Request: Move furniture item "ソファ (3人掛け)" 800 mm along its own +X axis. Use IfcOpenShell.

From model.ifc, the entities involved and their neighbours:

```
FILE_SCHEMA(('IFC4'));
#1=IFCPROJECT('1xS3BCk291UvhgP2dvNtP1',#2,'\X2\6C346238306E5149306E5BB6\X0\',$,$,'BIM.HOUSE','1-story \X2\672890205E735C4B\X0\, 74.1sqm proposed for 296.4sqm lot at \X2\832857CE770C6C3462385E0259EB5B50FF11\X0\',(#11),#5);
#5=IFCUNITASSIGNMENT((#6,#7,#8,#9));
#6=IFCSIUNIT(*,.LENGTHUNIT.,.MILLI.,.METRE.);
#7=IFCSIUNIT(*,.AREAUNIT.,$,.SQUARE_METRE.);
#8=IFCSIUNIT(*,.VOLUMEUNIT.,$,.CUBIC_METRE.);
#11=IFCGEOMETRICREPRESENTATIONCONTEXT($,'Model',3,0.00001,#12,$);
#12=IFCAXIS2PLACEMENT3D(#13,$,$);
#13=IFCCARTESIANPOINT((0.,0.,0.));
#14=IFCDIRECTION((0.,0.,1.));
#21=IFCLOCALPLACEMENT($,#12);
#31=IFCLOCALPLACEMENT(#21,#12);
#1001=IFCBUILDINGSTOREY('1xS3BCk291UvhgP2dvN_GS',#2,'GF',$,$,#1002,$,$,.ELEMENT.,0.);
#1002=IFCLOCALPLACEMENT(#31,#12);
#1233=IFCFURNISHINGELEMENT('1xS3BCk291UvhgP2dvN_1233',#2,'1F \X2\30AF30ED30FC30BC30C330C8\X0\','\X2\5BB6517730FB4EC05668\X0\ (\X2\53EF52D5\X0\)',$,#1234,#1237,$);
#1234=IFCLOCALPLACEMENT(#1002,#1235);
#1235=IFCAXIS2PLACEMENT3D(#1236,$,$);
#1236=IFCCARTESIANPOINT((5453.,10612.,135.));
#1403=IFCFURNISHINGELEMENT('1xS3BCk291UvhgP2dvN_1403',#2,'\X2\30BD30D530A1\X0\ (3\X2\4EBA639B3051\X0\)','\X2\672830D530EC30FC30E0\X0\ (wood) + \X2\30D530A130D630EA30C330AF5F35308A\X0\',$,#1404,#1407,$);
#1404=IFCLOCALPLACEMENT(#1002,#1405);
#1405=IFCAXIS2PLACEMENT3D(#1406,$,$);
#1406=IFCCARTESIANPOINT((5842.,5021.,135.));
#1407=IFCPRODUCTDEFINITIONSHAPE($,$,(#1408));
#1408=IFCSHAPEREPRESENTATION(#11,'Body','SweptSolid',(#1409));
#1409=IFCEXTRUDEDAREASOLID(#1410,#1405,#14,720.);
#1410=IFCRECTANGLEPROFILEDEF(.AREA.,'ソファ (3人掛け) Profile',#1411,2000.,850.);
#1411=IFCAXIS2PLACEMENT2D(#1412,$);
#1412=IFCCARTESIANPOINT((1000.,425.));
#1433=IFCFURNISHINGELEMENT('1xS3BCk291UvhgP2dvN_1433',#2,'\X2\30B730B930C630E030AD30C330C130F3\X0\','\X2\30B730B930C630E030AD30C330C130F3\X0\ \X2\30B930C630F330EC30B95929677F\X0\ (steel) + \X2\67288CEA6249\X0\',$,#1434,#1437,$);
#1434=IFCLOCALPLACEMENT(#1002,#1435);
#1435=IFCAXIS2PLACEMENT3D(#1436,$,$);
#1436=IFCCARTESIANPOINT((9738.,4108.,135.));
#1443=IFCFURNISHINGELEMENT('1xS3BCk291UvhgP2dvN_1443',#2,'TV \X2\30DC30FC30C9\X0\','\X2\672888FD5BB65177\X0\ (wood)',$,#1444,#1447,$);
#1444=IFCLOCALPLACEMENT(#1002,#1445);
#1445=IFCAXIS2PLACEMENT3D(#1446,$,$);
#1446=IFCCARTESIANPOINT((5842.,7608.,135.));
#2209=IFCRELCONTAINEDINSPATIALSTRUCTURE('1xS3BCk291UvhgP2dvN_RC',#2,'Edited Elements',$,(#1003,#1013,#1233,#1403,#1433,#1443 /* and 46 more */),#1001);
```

```python
import ifcopenshell
import ifcopenshell.api.geometry
import ifcopenshell.util.placement

model = ifcopenshell.open("model.ifc")

item = model.by_guid("1xS3BCk291UvhgP2dvN_1403")
matrix = ifcopenshell.util.placement.get_local_placement(item.ObjectPlacement)
matrix[:3, 3] += matrix[:3, 0] * 800.0
ifcopenshell.api.geometry.edit_object_placement(model, product=item, matrix=matrix, is_si=False)

print(ifcopenshell.util.placement.get_local_placement(item.ObjectPlacement).round(3) + 0.0)

model.write("model_rev.ifc")
```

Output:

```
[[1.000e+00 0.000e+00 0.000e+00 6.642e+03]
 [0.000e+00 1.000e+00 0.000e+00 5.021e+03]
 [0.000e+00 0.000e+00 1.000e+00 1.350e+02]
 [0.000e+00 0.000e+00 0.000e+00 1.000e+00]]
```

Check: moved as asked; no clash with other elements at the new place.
